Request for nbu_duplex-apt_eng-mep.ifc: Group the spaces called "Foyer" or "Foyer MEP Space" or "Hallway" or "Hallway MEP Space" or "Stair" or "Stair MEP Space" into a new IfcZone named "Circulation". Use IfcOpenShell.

First a look at what the model holds.

```python
import ifcopenshell

model = ifcopenshell.open("nbu_duplex-apt_eng-mep.ifc")
print(model.schema)
seen = {}
for space in model.by_type("IfcSpace"):
    seen[space.LongName] = seen.get(space.LongName, 0) + 1
for name, count in sorted(seen.items(), key=str):
    print(count, "x", name)
print("zones:", [z.Name for z in model.by_type("IfcZone")][:20])
```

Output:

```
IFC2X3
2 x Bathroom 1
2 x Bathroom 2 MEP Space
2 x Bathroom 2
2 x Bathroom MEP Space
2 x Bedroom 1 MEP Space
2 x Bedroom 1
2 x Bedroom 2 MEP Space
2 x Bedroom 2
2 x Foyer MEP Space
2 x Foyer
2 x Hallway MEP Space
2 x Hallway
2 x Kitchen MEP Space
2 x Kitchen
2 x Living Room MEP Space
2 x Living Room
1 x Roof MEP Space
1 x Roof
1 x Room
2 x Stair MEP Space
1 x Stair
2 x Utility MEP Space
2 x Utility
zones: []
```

```python
import ifcopenshell
import ifcopenshell.api.group
import ifcopenshell.api.root

model = ifcopenshell.open("nbu_duplex-apt_eng-mep.ifc")

names = {"Foyer", "Foyer MEP Space", "Hallway", "Hallway MEP Space", "Stair", "Stair MEP Space"}
spaces = [s for s in model.by_type("IfcSpace") if s.LongName in names]

zone = ifcopenshell.api.root.create_entity(model, ifc_class="IfcZone", name="Circulation")
ifcopenshell.api.group.assign_group(model, products=spaces, group=zone)
print(len(spaces), "spaces in", zone.Name)

model.write("nbu_duplex-apt_eng-mep_updated.ifc")
```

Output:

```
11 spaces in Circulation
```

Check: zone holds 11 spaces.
